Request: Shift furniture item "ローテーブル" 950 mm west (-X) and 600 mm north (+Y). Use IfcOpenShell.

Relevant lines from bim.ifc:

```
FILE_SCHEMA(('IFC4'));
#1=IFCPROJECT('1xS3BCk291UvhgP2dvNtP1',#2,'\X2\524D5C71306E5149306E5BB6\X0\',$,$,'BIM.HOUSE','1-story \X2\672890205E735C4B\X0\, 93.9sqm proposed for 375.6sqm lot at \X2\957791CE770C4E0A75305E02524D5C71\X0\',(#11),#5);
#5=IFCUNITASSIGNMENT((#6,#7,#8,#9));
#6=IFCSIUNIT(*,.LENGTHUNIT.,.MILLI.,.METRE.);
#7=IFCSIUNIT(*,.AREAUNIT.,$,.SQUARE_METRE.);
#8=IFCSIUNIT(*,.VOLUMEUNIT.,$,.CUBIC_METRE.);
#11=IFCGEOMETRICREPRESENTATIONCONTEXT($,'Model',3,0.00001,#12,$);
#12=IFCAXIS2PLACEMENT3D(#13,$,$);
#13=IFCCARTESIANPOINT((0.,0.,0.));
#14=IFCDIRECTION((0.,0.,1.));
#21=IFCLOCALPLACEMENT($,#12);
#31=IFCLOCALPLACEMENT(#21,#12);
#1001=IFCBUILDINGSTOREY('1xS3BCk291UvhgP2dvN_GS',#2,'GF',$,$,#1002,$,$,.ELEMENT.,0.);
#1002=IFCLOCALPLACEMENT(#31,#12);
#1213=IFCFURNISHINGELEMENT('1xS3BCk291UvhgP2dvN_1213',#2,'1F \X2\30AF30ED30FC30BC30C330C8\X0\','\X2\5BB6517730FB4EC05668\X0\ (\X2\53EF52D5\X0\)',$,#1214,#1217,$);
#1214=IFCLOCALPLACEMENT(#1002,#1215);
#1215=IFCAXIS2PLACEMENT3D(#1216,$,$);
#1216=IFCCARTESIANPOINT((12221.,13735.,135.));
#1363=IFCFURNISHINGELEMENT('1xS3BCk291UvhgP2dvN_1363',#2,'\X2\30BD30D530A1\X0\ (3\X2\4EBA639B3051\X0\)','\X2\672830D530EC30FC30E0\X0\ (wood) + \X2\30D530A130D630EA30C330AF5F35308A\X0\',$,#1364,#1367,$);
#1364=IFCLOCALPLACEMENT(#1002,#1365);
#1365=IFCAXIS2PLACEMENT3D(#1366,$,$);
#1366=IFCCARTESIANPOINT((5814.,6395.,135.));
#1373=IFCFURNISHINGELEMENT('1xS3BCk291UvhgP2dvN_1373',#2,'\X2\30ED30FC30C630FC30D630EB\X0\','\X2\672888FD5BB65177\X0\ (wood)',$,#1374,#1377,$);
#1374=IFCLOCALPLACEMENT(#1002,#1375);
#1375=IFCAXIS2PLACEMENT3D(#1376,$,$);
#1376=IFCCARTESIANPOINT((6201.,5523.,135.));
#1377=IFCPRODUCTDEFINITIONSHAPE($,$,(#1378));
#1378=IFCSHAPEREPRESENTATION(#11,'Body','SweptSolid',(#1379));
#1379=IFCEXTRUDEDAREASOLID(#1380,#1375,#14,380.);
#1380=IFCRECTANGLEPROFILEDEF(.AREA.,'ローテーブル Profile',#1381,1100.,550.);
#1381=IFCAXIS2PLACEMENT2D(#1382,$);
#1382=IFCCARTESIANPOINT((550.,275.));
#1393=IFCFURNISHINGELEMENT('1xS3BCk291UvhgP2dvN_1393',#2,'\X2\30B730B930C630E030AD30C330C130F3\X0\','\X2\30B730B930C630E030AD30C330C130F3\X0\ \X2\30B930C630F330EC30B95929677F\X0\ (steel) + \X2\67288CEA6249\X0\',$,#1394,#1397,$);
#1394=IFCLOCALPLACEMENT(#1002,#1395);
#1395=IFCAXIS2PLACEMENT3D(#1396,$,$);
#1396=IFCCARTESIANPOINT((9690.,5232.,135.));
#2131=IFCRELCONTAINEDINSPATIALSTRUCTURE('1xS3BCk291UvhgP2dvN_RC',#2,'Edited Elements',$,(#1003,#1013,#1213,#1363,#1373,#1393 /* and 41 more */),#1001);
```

```python
import ifcopenshell
import ifcopenshell.api.geometry
import ifcopenshell.util.placement

model = ifcopenshell.open("bim.ifc")

item = model.by_guid("1xS3BCk291UvhgP2dvN_1373")
matrix = ifcopenshell.util.placement.get_local_placement(item.ObjectPlacement)
matrix[0, 3] -= 950.0
matrix[1, 3] += 600.0
ifcopenshell.api.geometry.edit_object_placement(model, product=item, matrix=matrix, is_si=False)

print(ifcopenshell.util.placement.get_local_placement(item.ObjectPlacement).round(3) + 0.0)

model.write("bim_rev.ifc")
```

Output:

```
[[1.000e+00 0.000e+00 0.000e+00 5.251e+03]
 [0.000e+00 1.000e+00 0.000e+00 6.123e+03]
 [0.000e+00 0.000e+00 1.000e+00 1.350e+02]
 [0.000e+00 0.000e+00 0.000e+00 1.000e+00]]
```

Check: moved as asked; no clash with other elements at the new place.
